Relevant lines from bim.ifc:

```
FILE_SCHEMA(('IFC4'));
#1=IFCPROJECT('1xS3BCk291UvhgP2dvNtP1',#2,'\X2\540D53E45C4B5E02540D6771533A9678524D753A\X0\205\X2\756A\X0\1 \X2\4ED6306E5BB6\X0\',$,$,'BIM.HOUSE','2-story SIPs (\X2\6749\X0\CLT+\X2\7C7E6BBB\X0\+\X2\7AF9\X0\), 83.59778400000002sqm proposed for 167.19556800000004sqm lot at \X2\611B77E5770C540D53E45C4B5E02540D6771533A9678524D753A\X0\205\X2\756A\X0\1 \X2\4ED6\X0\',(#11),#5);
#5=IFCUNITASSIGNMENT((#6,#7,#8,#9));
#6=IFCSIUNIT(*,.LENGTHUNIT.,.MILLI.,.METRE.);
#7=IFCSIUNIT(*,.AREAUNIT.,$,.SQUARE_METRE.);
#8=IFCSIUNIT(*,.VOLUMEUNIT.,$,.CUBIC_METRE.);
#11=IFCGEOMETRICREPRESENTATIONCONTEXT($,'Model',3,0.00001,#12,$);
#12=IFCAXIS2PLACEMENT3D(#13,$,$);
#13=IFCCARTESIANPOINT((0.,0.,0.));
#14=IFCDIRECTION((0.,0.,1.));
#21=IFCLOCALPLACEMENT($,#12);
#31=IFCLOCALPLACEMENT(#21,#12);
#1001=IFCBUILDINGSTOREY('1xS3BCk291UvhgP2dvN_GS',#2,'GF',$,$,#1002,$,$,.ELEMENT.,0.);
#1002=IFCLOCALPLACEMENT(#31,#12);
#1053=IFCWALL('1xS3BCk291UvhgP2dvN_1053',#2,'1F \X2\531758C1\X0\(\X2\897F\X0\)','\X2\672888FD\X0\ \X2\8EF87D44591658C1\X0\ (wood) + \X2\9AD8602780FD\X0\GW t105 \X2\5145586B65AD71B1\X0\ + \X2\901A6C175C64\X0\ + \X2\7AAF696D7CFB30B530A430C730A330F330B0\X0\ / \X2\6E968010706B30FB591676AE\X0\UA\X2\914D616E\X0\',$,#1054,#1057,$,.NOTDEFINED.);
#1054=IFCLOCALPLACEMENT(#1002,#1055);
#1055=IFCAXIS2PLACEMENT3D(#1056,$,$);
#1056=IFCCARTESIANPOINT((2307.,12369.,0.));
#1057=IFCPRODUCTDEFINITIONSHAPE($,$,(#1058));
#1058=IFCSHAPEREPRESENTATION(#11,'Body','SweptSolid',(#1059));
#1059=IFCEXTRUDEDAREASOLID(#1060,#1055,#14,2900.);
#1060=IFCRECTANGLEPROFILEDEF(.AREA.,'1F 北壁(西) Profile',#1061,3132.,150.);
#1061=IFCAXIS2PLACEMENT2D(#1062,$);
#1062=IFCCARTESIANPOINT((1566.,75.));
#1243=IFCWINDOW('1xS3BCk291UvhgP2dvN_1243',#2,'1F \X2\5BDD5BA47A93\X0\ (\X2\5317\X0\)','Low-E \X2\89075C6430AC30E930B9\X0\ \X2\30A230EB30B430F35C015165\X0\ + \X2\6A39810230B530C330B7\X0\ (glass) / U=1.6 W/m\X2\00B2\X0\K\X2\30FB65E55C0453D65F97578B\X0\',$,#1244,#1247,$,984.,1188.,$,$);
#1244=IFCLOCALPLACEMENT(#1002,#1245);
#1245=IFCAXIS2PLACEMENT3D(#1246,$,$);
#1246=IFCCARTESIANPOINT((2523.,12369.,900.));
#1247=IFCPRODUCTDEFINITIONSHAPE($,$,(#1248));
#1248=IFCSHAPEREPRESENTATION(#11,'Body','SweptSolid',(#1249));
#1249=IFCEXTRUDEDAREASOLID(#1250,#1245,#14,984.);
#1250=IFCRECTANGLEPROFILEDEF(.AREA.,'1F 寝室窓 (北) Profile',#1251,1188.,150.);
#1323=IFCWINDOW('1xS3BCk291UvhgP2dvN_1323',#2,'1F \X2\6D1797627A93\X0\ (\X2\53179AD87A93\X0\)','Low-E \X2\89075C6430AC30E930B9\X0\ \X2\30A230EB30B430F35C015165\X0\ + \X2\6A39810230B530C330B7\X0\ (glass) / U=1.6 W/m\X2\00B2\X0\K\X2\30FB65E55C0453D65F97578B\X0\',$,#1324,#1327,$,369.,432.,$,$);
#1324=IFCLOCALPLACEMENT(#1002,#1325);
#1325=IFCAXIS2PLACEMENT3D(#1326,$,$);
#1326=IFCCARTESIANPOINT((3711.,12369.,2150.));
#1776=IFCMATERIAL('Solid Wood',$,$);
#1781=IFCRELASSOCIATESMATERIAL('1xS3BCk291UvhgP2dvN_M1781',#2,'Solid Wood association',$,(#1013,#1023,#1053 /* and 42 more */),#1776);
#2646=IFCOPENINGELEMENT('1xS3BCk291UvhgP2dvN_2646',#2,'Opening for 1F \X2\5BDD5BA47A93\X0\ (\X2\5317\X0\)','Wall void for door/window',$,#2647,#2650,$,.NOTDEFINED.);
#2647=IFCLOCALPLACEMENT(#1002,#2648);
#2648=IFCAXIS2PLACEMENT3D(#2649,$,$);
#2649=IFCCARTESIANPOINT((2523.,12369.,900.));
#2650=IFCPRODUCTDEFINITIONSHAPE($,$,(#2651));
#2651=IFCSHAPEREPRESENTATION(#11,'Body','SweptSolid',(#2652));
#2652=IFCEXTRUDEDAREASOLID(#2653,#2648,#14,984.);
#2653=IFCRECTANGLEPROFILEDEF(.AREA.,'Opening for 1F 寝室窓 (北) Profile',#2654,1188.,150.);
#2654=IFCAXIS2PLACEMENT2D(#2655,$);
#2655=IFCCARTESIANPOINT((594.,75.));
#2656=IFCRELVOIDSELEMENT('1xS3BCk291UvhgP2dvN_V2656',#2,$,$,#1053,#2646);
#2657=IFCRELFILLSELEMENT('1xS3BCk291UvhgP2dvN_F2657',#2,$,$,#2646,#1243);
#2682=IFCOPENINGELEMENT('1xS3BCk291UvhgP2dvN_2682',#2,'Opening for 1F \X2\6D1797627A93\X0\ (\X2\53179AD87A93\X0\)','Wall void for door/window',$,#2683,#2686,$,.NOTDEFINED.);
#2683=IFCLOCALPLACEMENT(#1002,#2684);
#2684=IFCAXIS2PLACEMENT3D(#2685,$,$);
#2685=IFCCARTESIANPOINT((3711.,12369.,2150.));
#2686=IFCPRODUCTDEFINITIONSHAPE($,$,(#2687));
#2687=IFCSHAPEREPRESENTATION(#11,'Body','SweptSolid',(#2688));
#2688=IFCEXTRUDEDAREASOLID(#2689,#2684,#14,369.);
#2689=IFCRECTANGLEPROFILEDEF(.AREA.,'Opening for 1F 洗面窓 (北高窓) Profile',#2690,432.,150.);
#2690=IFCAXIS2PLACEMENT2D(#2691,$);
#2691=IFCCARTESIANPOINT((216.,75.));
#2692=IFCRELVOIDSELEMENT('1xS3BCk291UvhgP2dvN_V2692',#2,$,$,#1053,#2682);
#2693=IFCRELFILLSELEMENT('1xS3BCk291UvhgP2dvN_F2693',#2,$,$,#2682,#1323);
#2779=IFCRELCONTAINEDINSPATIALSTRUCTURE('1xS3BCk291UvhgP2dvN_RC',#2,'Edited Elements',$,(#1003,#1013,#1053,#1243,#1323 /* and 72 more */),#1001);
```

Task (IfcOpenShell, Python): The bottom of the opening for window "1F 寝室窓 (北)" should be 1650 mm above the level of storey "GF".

```python
import numpy as np
import ifcopenshell
import ifcopenshell.api.geometry
import ifcopenshell.geom
import ifcopenshell.util.element
import ifcopenshell.util.placement
import ifcopenshell.util.shape
import ifcopenshell.util.unit

model = ifcopenshell.open("bim.ifc")
unit_scale = ifcopenshell.util.unit.calculate_unit_scale(model)

window = model.by_guid("1xS3BCk291UvhgP2dvN_1243")
opening = window.FillsVoids[0].RelatingOpeningElement
storey = ifcopenshell.util.element.get_container(window, ifc_class="IfcBuildingStorey")
level = ifcopenshell.util.placement.get_local_placement(storey.ObjectPlacement)[2, 3]

# The opening's origin need not be at the sill, so measure its lowest point.
shape = ifcopenshell.geom.create_shape(ifcopenshell.geom.settings(), opening)
bottom = ifcopenshell.util.shape.get_shape_bottom_elevation(shape, shape.geometry) / unit_scale
dz = level + 1650.0 - bottom

shift = np.array([0.0, 0.0, dz])
# The window is not placed relative to its opening, so move both.
for product in (opening, window):
    matrix = ifcopenshell.util.placement.get_local_placement(product.ObjectPlacement)
    matrix[:3, 3] += shift
    ifcopenshell.api.geometry.edit_object_placement(model, product=product, matrix=matrix, is_si=False)

print(f"moved by {dz * unit_scale:+.3f} m")

model.write("bim-out.ifc")
```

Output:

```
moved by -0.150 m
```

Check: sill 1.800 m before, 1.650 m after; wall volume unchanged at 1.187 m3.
